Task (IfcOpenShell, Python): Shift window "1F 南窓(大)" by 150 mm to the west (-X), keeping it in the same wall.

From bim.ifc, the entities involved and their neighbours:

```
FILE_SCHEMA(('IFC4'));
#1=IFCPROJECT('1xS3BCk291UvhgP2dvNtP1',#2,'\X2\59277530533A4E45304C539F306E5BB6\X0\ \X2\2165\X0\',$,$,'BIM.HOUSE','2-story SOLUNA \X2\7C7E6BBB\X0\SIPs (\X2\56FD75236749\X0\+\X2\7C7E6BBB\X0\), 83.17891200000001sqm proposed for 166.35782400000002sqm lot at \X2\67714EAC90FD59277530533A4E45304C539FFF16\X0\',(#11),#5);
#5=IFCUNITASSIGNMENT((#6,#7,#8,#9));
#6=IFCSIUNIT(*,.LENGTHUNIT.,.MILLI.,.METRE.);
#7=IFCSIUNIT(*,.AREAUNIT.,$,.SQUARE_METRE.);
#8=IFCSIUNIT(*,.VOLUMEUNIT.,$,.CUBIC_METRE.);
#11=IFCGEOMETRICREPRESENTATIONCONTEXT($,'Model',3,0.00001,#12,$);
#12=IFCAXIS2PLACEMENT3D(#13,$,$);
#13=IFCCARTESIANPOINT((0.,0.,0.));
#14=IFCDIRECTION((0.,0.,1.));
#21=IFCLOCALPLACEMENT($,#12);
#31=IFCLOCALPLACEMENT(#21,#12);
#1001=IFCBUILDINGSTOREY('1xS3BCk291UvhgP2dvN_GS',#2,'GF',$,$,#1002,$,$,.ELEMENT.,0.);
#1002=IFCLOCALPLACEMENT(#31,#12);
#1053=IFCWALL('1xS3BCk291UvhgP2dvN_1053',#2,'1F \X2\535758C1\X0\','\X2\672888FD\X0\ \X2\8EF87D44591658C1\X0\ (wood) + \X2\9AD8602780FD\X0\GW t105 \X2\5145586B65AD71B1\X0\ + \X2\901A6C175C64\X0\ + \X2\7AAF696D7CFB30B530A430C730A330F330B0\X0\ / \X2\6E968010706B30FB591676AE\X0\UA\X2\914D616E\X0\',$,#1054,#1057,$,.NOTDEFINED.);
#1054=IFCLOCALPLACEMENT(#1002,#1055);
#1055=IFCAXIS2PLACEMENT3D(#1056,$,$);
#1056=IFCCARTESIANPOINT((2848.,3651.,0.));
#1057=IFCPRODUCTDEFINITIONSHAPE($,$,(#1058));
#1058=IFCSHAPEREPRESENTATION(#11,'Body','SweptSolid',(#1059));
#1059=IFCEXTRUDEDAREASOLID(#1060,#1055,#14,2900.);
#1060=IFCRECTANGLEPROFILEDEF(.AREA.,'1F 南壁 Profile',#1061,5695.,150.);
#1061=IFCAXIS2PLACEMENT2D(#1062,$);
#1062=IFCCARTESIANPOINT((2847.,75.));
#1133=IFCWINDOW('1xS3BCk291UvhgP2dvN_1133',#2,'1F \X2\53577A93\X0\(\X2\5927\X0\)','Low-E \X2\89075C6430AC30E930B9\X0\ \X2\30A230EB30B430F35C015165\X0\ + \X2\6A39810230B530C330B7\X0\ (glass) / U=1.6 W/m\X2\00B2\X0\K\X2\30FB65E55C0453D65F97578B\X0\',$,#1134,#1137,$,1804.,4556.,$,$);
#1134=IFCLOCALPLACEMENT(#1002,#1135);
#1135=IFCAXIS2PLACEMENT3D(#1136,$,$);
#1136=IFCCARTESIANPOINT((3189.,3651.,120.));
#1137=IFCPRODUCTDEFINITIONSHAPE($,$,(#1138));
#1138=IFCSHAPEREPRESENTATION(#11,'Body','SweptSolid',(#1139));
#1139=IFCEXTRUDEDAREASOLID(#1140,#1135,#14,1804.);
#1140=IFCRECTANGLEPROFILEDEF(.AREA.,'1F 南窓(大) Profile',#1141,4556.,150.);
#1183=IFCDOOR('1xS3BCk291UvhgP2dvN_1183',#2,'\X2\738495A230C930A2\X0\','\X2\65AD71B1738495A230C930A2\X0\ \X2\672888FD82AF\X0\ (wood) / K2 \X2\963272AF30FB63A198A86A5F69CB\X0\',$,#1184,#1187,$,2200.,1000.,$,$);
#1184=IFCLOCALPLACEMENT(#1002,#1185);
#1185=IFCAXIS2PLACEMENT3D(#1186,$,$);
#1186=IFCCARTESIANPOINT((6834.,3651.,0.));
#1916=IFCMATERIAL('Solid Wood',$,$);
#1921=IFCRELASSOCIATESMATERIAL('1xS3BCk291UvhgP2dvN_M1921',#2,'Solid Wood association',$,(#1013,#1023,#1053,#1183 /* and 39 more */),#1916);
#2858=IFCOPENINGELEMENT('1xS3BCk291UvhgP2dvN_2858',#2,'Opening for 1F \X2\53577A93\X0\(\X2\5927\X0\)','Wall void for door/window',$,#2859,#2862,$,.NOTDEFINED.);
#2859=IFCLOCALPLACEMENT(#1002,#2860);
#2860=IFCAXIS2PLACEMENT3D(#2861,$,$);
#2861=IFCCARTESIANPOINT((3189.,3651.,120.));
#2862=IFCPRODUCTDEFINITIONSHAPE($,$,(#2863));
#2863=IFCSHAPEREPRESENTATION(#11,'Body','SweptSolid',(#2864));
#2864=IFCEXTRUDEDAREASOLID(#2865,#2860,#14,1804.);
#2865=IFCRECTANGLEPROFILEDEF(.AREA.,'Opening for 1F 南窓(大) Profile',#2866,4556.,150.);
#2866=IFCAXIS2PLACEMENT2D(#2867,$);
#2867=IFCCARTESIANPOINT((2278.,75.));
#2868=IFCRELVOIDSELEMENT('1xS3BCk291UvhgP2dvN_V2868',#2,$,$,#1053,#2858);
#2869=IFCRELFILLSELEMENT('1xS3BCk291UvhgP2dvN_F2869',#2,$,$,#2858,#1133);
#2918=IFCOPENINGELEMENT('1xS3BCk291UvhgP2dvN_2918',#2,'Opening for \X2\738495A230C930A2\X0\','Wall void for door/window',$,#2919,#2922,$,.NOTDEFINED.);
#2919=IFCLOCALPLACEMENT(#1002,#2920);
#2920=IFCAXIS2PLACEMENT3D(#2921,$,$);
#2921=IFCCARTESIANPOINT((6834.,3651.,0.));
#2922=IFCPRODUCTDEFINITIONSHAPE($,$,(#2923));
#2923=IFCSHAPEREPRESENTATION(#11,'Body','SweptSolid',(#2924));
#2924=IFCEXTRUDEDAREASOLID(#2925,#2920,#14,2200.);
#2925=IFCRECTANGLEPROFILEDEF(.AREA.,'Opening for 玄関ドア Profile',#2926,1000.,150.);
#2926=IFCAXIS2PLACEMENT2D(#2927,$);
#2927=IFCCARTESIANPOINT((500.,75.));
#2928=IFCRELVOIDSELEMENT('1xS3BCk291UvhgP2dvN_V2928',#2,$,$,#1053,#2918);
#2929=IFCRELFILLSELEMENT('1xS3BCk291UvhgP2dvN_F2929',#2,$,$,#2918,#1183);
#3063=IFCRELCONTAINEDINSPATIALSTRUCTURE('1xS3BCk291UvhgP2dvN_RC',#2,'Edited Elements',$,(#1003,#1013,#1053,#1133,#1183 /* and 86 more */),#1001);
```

```python
import ifcopenshell
import ifcopenshell.api.geometry
import ifcopenshell.util.placement
import ifcopenshell.util.unit

model = ifcopenshell.open("bim.ifc")
unit_scale = ifcopenshell.util.unit.calculate_unit_scale(model)

window = model.by_guid("1xS3BCk291UvhgP2dvN_1133")
opening = window.FillsVoids[0].RelatingOpeningElement
wall = opening.VoidsElements[0].RelatingBuildingElement

wall_matrix = ifcopenshell.util.placement.get_local_placement(wall.ObjectPlacement)
shift = wall_matrix[:3, 0] * -0.15 / unit_scale
before = ifcopenshell.util.placement.get_local_placement(window.ObjectPlacement)[:3, 3].copy()

# The window is not placed relative to its opening, so move both.
for product in (opening, window):
    matrix = ifcopenshell.util.placement.get_local_placement(product.ObjectPlacement)
    matrix[:3, 3] += shift
    ifcopenshell.api.geometry.edit_object_placement(model, product=product, matrix=matrix, is_si=False)

after = ifcopenshell.util.placement.get_local_placement(window.ObjectPlacement)[:3, 3]
print("window moved by", (after - before).round(3) + 0.0)

model.write("bim_v2.ifc")
```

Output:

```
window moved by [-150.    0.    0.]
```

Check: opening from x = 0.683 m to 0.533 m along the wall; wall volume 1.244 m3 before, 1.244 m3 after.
